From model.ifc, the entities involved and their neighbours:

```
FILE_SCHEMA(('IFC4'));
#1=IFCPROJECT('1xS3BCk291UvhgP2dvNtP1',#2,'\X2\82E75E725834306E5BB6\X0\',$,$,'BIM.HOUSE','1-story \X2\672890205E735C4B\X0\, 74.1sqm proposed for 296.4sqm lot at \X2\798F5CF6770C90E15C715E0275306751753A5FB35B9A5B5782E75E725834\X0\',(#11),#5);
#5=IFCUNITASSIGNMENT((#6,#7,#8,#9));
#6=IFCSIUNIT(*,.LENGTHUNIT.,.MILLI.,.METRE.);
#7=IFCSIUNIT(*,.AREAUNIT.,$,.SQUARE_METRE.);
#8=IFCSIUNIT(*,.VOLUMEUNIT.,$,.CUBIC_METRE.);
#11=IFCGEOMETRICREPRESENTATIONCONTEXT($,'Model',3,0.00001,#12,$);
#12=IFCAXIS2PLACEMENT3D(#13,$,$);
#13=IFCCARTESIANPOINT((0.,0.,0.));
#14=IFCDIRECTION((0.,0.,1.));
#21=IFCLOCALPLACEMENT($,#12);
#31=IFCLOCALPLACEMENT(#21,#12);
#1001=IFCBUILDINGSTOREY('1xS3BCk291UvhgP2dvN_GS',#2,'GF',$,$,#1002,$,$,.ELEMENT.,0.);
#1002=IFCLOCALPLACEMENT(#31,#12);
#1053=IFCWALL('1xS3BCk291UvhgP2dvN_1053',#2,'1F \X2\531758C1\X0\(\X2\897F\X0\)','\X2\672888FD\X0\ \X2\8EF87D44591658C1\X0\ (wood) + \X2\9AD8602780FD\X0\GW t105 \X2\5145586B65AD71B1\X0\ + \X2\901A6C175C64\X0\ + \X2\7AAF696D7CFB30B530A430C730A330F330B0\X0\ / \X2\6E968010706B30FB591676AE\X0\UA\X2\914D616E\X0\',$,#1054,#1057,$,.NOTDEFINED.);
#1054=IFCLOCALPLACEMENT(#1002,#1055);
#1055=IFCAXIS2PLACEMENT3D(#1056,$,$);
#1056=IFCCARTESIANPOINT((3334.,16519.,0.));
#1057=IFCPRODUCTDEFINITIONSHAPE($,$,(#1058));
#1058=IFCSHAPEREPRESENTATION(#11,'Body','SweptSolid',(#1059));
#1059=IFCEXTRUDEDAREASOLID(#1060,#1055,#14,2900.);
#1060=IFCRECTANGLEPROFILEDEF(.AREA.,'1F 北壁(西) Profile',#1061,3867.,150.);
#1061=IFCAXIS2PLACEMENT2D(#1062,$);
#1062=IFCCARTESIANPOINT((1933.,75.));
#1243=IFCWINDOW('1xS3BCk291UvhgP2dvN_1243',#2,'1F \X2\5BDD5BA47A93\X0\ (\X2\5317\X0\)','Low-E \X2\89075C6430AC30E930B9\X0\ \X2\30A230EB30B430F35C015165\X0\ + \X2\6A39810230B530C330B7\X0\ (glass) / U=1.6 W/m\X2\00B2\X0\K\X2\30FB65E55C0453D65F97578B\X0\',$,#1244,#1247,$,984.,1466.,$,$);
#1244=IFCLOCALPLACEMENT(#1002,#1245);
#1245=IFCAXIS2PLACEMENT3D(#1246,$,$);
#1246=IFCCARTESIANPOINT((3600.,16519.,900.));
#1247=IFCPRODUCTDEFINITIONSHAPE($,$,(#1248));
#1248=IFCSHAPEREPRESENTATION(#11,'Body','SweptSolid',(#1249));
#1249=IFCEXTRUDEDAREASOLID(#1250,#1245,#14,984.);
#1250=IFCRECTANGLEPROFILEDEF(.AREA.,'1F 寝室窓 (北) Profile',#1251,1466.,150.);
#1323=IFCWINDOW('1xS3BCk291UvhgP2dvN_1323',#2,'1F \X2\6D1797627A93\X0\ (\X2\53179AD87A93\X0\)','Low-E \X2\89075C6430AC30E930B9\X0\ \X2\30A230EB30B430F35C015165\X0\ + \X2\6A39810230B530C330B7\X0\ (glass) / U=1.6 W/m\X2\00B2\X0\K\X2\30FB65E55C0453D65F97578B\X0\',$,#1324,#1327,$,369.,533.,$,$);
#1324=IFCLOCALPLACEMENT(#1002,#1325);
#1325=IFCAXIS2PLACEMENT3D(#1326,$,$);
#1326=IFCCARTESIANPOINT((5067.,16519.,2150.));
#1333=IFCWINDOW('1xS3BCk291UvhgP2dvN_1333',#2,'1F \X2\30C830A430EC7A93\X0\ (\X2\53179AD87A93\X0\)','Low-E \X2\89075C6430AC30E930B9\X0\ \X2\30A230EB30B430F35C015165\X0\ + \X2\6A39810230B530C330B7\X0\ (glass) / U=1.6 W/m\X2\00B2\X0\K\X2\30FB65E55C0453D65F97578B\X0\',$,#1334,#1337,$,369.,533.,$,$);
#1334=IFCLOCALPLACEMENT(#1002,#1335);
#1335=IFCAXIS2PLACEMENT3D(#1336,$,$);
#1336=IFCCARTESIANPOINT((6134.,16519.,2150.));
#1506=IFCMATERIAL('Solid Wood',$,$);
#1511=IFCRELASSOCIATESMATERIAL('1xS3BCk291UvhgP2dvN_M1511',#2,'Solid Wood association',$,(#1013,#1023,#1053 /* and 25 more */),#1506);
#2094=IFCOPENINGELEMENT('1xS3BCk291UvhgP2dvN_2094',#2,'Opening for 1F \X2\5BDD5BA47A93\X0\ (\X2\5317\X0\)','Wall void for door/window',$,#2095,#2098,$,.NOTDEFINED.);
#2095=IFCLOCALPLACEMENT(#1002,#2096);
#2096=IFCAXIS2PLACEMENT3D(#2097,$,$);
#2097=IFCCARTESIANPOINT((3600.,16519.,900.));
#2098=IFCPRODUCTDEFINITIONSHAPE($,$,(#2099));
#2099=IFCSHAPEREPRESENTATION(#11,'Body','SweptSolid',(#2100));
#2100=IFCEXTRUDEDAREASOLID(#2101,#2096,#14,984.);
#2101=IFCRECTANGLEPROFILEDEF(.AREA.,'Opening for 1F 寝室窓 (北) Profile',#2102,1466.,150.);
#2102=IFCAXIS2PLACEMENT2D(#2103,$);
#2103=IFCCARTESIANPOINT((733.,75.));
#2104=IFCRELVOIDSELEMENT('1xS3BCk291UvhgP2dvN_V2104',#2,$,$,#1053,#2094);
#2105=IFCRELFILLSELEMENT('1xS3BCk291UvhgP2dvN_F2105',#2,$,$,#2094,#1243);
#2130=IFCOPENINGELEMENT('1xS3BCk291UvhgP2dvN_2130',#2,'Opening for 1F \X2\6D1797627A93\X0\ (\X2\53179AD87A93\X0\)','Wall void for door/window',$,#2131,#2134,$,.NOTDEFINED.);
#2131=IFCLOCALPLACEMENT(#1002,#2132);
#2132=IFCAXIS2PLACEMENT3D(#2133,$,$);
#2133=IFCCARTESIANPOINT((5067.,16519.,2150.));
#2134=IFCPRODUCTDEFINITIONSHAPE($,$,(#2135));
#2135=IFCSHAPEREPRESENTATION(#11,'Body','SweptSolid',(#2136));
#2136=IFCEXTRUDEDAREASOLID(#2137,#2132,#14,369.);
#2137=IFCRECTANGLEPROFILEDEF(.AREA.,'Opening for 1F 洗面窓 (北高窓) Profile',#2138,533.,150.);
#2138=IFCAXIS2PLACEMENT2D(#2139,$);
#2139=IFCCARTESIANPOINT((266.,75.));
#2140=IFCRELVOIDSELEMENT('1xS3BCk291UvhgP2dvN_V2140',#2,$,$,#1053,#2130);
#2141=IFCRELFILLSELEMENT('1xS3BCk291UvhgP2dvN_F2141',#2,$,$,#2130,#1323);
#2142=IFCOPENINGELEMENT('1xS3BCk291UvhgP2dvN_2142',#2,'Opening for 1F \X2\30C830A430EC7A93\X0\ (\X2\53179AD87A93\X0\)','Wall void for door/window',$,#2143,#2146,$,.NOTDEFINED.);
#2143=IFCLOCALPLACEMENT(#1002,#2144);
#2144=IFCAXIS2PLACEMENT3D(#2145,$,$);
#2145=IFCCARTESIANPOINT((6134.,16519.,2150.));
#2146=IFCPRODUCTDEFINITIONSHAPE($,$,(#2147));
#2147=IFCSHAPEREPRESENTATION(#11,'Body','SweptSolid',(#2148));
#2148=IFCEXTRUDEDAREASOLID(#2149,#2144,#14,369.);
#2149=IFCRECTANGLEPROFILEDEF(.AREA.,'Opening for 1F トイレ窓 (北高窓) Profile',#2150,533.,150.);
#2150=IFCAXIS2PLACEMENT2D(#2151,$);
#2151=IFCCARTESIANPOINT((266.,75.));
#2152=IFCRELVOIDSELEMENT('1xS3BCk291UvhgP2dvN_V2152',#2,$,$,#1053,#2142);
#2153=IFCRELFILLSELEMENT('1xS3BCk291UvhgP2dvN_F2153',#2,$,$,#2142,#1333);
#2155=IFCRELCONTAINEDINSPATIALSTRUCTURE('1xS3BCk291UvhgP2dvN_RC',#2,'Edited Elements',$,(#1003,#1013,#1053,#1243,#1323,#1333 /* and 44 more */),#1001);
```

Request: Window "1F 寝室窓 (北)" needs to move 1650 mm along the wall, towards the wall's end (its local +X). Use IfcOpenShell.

```python
import ifcopenshell
import ifcopenshell.api.geometry
import ifcopenshell.util.placement
import ifcopenshell.util.unit

model = ifcopenshell.open("model.ifc")
unit_scale = ifcopenshell.util.unit.calculate_unit_scale(model)

window = model.by_guid("1xS3BCk291UvhgP2dvN_1243")
opening = window.FillsVoids[0].RelatingOpeningElement
wall = opening.VoidsElements[0].RelatingBuildingElement

wall_matrix = ifcopenshell.util.placement.get_local_placement(wall.ObjectPlacement)
shift = wall_matrix[:3, 0] * 1.65 / unit_scale
before = ifcopenshell.util.placement.get_local_placement(window.ObjectPlacement)[:3, 3].copy()

# The window is not placed relative to its opening, so move both.
for product in (opening, window):
    matrix = ifcopenshell.util.placement.get_local_placement(product.ObjectPlacement)
    matrix[:3, 3] += shift
    ifcopenshell.api.geometry.edit_object_placement(model, product=product, matrix=matrix, is_si=False)

after = ifcopenshell.util.placement.get_local_placement(window.ObjectPlacement)[:3, 3]
print("window moved by", (after - before).round(3) + 0.0)

model.write("model_v2.ifc")
```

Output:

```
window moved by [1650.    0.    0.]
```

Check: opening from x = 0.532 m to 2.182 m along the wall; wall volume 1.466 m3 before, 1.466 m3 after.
